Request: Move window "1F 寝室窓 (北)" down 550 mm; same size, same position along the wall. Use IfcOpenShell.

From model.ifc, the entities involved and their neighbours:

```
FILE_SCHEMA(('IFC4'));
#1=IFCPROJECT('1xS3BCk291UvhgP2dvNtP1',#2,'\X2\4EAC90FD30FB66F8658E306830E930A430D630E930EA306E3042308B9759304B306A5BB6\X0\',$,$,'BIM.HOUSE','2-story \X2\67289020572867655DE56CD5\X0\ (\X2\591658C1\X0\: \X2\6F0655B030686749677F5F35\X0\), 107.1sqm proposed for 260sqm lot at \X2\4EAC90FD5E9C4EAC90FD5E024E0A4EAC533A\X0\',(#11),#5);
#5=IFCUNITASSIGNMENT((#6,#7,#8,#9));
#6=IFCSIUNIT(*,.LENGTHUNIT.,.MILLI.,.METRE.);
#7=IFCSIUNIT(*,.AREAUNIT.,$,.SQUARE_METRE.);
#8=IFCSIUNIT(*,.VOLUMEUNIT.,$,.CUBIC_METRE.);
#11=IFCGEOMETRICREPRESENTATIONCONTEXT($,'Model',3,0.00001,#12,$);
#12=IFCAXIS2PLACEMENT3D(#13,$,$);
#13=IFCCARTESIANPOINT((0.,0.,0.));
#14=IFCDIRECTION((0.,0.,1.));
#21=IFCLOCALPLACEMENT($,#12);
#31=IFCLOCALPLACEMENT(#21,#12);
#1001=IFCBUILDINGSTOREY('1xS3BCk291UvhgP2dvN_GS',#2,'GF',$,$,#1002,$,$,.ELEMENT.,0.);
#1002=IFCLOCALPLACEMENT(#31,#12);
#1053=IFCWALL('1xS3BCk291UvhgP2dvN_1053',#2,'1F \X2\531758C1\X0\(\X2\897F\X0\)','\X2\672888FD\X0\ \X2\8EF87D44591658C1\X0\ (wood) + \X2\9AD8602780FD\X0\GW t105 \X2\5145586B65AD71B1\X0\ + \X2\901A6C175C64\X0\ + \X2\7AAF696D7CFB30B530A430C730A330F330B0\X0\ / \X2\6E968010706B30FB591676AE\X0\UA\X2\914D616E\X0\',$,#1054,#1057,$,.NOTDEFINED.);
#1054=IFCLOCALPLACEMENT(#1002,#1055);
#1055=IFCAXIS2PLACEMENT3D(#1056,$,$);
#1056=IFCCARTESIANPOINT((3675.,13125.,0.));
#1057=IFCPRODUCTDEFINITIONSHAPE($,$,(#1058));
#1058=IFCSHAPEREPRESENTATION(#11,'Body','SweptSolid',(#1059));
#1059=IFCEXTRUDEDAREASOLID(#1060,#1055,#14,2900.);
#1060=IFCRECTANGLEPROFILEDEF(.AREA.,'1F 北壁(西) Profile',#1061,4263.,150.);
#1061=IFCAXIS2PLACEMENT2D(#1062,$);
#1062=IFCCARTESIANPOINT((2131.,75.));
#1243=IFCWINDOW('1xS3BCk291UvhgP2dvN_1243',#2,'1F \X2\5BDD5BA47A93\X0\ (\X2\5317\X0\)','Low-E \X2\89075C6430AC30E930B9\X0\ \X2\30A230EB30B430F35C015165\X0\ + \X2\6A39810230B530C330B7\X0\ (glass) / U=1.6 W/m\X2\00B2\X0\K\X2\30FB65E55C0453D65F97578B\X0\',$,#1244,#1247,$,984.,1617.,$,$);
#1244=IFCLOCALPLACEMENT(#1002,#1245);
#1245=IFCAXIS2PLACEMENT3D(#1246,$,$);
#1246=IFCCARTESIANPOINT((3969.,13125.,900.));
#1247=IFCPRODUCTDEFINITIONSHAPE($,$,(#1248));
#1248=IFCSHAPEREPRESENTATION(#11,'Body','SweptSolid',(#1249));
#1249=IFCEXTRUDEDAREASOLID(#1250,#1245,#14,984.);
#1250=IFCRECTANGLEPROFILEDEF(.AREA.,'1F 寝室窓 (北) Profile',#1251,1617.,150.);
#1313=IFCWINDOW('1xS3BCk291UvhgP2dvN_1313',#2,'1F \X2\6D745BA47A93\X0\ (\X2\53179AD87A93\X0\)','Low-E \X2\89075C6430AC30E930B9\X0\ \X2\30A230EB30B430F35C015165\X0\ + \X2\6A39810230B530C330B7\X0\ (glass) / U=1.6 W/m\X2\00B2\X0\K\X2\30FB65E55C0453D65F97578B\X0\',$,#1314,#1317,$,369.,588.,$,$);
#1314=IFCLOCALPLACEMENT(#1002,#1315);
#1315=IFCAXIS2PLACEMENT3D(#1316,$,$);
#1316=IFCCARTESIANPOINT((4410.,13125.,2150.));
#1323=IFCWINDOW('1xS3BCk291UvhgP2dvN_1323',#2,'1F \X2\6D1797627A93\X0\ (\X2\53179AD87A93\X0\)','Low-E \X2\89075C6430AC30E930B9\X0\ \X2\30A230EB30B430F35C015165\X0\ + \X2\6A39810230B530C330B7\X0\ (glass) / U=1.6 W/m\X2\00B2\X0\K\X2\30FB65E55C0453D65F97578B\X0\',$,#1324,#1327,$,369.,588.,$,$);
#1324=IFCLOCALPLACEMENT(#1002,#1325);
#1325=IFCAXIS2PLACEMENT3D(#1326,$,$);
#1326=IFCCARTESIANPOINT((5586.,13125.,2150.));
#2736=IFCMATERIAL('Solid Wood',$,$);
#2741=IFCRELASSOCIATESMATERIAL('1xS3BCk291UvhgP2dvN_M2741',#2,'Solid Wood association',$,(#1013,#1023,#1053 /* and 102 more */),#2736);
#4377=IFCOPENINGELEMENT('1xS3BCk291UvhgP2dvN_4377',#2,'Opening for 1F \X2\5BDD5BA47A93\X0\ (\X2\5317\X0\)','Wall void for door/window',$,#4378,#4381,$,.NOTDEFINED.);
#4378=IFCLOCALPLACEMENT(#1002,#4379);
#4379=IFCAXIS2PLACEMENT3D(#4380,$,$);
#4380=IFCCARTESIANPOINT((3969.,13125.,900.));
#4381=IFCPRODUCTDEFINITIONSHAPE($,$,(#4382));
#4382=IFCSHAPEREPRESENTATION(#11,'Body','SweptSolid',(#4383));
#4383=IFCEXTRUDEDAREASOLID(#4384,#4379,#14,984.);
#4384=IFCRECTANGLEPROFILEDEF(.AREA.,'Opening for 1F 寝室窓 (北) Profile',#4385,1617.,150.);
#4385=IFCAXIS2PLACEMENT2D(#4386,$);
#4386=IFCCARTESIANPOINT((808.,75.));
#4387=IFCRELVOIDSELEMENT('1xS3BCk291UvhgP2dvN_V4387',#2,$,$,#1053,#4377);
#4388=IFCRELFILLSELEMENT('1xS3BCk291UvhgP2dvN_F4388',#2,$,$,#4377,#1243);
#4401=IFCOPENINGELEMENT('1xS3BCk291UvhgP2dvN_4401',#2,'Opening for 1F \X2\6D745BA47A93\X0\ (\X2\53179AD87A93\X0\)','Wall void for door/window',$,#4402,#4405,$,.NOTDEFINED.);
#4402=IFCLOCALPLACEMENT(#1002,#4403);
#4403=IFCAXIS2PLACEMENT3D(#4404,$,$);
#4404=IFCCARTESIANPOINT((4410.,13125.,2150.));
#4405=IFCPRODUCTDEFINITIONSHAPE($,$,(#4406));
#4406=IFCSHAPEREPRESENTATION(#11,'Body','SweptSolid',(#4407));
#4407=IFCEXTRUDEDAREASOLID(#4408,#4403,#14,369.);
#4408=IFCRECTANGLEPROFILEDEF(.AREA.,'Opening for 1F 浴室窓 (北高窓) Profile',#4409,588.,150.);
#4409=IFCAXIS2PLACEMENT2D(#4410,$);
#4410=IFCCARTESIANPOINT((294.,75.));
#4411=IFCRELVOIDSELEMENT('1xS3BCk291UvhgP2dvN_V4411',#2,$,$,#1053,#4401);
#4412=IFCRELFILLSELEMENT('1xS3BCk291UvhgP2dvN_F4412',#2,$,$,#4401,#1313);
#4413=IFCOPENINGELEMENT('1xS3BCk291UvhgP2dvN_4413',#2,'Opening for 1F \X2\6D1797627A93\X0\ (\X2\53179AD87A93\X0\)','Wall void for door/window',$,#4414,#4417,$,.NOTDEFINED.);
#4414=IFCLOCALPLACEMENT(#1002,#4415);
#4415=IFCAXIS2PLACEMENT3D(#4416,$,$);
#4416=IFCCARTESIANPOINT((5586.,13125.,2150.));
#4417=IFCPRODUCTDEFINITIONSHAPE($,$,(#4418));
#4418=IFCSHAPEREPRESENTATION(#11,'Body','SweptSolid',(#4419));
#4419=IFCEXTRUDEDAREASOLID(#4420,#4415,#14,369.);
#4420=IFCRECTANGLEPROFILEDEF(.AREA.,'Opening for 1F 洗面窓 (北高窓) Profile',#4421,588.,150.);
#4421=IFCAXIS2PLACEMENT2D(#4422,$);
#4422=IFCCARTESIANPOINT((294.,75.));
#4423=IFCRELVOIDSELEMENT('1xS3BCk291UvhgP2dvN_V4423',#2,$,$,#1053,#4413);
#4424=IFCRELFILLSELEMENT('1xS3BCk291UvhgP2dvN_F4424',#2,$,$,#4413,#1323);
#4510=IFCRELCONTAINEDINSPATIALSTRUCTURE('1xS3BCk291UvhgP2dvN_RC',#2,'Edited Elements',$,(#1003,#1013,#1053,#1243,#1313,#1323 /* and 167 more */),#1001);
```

```python
import numpy as np
import ifcopenshell
import ifcopenshell.api.geometry
import ifcopenshell.util.placement
import ifcopenshell.util.unit

model = ifcopenshell.open("model.ifc")
unit_scale = ifcopenshell.util.unit.calculate_unit_scale(model)

window = model.by_guid("1xS3BCk291UvhgP2dvN_1243")
opening = window.FillsVoids[0].RelatingOpeningElement
dz = -550.0

shift = np.array([0.0, 0.0, dz])
# The window is not placed relative to its opening, so move both.
for product in (opening, window):
    matrix = ifcopenshell.util.placement.get_local_placement(product.ObjectPlacement)
    matrix[:3, 3] += shift
    ifcopenshell.api.geometry.edit_object_placement(model, product=product, matrix=matrix, is_si=False)

print(f"moved by {dz * unit_scale:+.3f} m")

model.write("model_updated.ifc")
```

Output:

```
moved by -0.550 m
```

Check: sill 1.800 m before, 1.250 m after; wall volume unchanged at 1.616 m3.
